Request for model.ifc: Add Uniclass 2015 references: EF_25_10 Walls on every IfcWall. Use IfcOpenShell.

First a look at what the model holds.

```python
import ifcopenshell

model = ifcopenshell.open("model.ifc")
print(model.schema)
print("classifications:", [c.Name for c in model.by_type("IfcClassification")])
for ifc_class in ("IfcDoor", "IfcRoof", "IfcStair", "IfcWall", "IfcWindow"):
    print(ifc_class, len(model.by_type(ifc_class)))
```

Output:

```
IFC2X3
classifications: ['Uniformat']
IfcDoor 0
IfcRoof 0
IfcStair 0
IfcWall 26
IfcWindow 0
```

```python
import ifcopenshell
import ifcopenshell.api.classification

model = ifcopenshell.open("model.ifc")

# IFC2X3 requires Source and Edition and has no link from the project to the system.
system = model.create_entity("IfcClassification", Source="NBS", Edition="2015", Name="Uniclass 2015")

codes = {
    "IfcWall": ("EF_25_10", "Walls"),
}
for ifc_class, (code, name) in codes.items():
    products = model.by_type(ifc_class)
    ifcopenshell.api.classification.add_reference(
        model, products=products, classification=system, identification=code, name=name
    )
    print(code, len(products))

model.write("model_rev.ifc")
```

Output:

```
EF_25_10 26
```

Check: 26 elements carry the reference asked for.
